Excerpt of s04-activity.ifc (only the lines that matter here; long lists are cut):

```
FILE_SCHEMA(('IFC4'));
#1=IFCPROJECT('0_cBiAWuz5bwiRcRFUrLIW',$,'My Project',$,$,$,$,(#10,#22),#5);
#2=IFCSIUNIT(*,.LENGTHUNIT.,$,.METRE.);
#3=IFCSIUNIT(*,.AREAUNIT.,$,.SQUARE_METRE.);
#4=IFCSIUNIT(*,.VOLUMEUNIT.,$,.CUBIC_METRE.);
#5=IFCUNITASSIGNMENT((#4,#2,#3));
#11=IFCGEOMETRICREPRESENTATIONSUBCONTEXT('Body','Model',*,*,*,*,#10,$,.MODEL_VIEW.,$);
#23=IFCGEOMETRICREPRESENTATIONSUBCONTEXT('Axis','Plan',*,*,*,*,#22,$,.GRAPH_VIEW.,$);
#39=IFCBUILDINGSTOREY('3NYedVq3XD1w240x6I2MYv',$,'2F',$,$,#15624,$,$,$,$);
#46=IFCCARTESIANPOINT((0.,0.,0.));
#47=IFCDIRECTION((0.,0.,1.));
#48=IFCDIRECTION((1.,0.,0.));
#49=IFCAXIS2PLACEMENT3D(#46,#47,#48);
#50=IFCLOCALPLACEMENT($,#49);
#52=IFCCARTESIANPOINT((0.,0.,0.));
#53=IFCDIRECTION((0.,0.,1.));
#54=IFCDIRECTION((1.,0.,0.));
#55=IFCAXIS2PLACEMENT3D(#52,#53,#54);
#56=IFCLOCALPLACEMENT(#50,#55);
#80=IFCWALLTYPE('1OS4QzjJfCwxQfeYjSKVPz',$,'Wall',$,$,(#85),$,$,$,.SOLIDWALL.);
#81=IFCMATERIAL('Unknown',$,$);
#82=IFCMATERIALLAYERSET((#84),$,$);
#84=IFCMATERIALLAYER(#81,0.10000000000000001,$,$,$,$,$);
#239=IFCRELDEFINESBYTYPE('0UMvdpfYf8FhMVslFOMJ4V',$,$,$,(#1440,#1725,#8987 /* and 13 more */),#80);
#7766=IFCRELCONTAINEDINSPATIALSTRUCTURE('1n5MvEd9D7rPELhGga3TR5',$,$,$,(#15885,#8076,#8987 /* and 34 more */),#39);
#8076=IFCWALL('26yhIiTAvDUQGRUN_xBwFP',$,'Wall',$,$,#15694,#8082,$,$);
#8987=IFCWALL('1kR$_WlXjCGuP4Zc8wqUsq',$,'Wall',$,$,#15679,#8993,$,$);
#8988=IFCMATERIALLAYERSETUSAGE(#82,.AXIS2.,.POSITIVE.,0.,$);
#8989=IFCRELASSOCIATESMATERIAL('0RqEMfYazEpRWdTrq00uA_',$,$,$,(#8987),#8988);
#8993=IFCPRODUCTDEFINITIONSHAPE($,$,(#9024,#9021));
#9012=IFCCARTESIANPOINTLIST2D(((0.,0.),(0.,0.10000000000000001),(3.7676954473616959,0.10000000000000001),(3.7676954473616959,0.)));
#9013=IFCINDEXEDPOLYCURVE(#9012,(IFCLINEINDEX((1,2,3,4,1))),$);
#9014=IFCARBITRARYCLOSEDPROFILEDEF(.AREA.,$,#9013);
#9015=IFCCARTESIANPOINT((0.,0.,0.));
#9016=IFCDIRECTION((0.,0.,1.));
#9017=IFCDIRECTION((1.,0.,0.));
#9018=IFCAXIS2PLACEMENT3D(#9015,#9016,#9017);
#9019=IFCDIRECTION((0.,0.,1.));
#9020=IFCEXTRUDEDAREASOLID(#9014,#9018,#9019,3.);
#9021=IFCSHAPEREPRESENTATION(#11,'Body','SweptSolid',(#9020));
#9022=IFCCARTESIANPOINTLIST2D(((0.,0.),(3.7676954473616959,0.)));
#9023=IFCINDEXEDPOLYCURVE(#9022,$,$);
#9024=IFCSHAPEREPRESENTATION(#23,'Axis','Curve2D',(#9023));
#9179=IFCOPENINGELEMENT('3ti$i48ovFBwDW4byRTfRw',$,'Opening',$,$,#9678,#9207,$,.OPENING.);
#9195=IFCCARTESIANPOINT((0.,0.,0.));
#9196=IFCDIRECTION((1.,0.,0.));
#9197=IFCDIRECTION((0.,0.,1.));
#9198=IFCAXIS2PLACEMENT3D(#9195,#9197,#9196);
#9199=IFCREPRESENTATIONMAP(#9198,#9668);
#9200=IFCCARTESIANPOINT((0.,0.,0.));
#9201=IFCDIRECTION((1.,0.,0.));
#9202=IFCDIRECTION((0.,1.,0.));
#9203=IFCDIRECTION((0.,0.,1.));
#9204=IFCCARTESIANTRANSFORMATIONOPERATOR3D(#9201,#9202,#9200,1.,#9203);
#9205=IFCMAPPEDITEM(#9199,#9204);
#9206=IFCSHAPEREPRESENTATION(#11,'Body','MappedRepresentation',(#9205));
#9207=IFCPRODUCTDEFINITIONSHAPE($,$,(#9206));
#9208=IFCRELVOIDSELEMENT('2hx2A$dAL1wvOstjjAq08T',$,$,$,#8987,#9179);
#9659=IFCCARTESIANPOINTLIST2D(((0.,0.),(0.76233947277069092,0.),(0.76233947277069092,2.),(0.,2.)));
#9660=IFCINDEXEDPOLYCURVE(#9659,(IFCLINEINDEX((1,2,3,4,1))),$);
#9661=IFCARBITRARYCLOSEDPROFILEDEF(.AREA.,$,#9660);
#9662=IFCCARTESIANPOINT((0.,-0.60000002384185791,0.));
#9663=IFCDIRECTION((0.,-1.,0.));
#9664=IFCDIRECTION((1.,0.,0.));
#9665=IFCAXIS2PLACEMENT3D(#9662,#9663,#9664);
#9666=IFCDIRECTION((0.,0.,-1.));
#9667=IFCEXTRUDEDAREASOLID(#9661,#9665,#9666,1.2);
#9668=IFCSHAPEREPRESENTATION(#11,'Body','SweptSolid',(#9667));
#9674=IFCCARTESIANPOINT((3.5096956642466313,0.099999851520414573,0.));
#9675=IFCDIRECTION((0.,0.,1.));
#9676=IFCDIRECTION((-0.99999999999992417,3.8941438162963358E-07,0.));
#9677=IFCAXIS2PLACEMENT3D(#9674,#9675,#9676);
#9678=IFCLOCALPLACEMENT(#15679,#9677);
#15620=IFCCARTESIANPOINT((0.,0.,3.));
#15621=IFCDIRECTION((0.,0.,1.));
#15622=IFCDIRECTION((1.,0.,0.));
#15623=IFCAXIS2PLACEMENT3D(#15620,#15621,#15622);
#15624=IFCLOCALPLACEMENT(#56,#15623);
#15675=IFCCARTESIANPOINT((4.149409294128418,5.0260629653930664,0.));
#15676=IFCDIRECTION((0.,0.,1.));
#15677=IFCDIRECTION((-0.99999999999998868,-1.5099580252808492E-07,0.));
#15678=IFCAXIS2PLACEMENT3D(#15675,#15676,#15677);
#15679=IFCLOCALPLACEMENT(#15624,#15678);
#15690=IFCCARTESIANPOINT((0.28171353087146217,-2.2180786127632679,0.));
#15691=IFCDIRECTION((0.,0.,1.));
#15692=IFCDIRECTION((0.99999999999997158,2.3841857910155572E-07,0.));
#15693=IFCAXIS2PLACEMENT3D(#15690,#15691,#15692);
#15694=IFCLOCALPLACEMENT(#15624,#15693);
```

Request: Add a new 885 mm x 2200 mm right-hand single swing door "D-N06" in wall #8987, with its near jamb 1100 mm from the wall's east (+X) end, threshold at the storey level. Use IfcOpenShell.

```python
import numpy as np
import ifcopenshell
import ifcopenshell.api.feature
import ifcopenshell.api.geometry
import ifcopenshell.api.root
import ifcopenshell.api.spatial
import ifcopenshell.geom
import ifcopenshell.util.element
import ifcopenshell.util.placement
import ifcopenshell.util.representation
import ifcopenshell.util.shape
import ifcopenshell.util.unit

model = ifcopenshell.open("s04-activity.ifc")
unit_scale = ifcopenshell.util.unit.calculate_unit_scale(model)
settings = ifcopenshell.geom.settings()


def volume(element):
    """Net volume in cubic metres, openings subtracted."""
    shape = ifcopenshell.geom.create_shape(settings, element)
    return ifcopenshell.util.shape.get_volume(shape.geometry)


wall = model.by_guid("1kR$_WlXjCGuP4Zc8wqUsq")
storey = ifcopenshell.util.element.get_container(wall, ifc_class="IfcBuildingStorey")
context = ifcopenshell.util.representation.get_context(model, "Model", "Body", "MODEL_VIEW")
before = volume(wall)

width, height, from_end, sill = 0.885, 2.2, 1.1, 0.0  # metres

# The wall runs along its own X axis, and the end named is its -X end.
wall_shape = ifcopenshell.geom.create_shape(settings, wall)
x, y, z = ifcopenshell.util.shape.get_vertices(wall_shape.geometry).T
start = x.min() + from_end
face, thickness = float(y.min()), float(y.max() - y.min())
wall_matrix = ifcopenshell.util.placement.get_local_placement(wall.ObjectPlacement)
level = ifcopenshell.util.placement.get_local_placement(storey.ObjectPlacement)[2, 3]


def in_wall(x, y):
    """Placement at x, y metres in the wall's axes, at sill height."""
    matrix = wall_matrix.copy()
    matrix[:, 3] = wall_matrix @ np.array([x / unit_scale, y / unit_scale, 0.0, 1.0])
    matrix[2, 3] = level + sill / unit_scale
    return matrix


# Opening: a box that overshoots both wall faces by 50 mm.
opening = ifcopenshell.api.root.create_entity(model, ifc_class="IfcOpeningElement", predefined_type="OPENING")
box = ifcopenshell.api.geometry.add_wall_representation(
    model, context=context, length=width, height=height, thickness=thickness + 0.1
)
ifcopenshell.api.geometry.assign_representation(model, product=opening, representation=box)
ifcopenshell.api.geometry.edit_object_placement(model, product=opening, matrix=in_wall(start, face - 0.05), is_si=False)
ifcopenshell.api.feature.add_feature(model, feature=opening, element=wall)

door = ifcopenshell.api.root.create_entity(model, ifc_class="IfcDoor", name="D-N06", predefined_type="DOOR")
door.OverallWidth, door.OverallHeight = width / unit_scale, height / unit_scale
door.OperationType = "SINGLE_SWING_RIGHT"
body = ifcopenshell.api.geometry.add_door_representation(
    model,
    context=context,
    overall_width=door.OverallWidth,
    overall_height=door.OverallHeight,
    operation_type="SINGLE_SWING_RIGHT",
    lining_properties={"LiningDepth": thickness / unit_scale, "ThresholdDepth": thickness / unit_scale},
)
ifcopenshell.api.geometry.assign_representation(model, product=door, representation=body)
ifcopenshell.api.spatial.assign_container(model, products=[door], relating_structure=storey)
ifcopenshell.api.feature.add_filling(model, opening=opening, element=door)

# The lining spans the wall, so the door starts at the wall face.
ifcopenshell.api.geometry.edit_object_placement(model, product=door, matrix=in_wall(start, face), is_si=False)

after = volume(wall)

print(f"wall volume {before:.3f} -> {after:.3f} m3")

model.write("s04-activity-out.ifc")
```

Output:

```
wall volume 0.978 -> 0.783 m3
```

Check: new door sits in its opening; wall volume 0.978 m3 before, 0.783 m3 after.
